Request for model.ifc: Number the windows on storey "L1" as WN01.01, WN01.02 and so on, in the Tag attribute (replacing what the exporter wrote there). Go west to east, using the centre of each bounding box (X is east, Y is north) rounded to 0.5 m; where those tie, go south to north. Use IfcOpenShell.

First a look at what the model holds.

```python
import ifcopenshell
import ifcopenshell.util.element
import ifcopenshell.util.placement

model = ifcopenshell.open("model.ifc")
print(model.schema)
storey = next(s for s in model.by_type("IfcBuildingStorey") if s.Name == "L1")
windows = [e for e in ifcopenshell.util.element.get_decomposition(storey) if e.is_a("IfcWindow")]
for e in sorted(windows, key=lambda e: e.id()):
    origin = ifcopenshell.util.placement.get_local_placement(e.ObjectPlacement)[:3, 3]
    print(e.id(), e.Tag, e.Name, origin.round(2) + 0.0, sep=" | ")
```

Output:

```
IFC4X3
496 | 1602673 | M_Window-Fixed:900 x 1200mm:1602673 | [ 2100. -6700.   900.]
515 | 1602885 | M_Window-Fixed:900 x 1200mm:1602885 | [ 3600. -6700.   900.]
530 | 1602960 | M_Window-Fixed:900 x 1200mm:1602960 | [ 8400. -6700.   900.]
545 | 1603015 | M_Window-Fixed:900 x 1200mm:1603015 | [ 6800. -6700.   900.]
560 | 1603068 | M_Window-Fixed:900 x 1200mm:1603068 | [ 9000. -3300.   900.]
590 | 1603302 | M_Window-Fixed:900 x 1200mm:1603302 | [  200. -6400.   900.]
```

```python
import ifcopenshell
import ifcopenshell.geom
import ifcopenshell.util.element
import ifcopenshell.util.shape

model = ifcopenshell.open("model.ifc")
settings = ifcopenshell.geom.settings()
settings.set("use-world-coords", True)


def centre(element):
    shape = ifcopenshell.geom.create_shape(settings, element)
    return ifcopenshell.util.shape.get_bbox_centroid(shape.geometry)


storey = next(s for s in model.by_type("IfcBuildingStorey") if s.Name == "L1")
windows = [e for e in ifcopenshell.util.element.get_decomposition(storey) if e.is_a("IfcWindow")]

# Insertion points can sit at a corner or the storey origin, so sort by the geometry (in metres).
centres = {e: centre(e) for e in windows}
windows.sort(key=lambda e: (round(centres[e][0] / 0.5), centres[e][1]))

for i, e in enumerate(windows, start=1):
    number = f"WN01.{i:02d}"
    e.Tag = number
    print(e.id(), number)

model.write("model-out.ifc")
```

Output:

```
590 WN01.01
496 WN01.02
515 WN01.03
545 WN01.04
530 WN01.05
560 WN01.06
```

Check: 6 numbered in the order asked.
